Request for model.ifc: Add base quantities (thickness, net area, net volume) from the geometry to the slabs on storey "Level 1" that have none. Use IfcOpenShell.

First a look at what the model holds.

```python
import ifcopenshell
import ifcopenshell.util.element
import ifcopenshell.util.unit

model = ifcopenshell.open("model.ifc")
print(model.schema)
for unit_type in ("LENGTHUNIT", "AREAUNIT", "VOLUMEUNIT"):
    print(unit_type, ifcopenshell.util.unit.calculate_unit_scale(model, unit_type))
storey = next(s for s in model.by_type("IfcBuildingStorey") if s.Name == "Level 1")
slabs = [e for e in ifcopenshell.util.element.get_decomposition(storey) if e.is_a("IfcSlab")]
for e in sorted(slabs, key=lambda e: e.id()):
    print(e.id(), e.is_a(), e.Name, list(ifcopenshell.util.element.get_psets(e, qtos_only=True)), sep=" | ")
```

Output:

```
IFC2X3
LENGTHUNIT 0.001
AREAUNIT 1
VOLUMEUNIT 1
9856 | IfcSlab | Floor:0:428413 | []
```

```python
import ifcopenshell
import ifcopenshell.api.pset
import ifcopenshell.geom
import ifcopenshell.util.element
import ifcopenshell.util.shape
import ifcopenshell.util.unit

model = ifcopenshell.open("model.ifc")
unit_scale = ifcopenshell.util.unit.calculate_unit_scale(model)
area_scale = ifcopenshell.util.unit.calculate_unit_scale(model, "AREAUNIT")
volume_scale = ifcopenshell.util.unit.calculate_unit_scale(model, "VOLUMEUNIT")
settings = ifcopenshell.geom.settings()

storey = next(s for s in model.by_type("IfcBuildingStorey") if s.Name == "Level 1")
slabs = [e for e in ifcopenshell.util.element.get_decomposition(storey) if e.is_a("IfcSlab")]

for e in sorted(slabs, key=lambda e: e.id()):
    if ifcopenshell.util.element.get_psets(e, qtos_only=True, should_inherit=False):
        continue
    # Geometry comes back in metres, in the element's own axes.
    shape = ifcopenshell.geom.create_shape(settings, e)
    values = {
        "Width": ifcopenshell.util.shape.get_z(shape.geometry) / unit_scale,
        "NetArea": ifcopenshell.util.shape.get_footprint_area(shape.geometry) / area_scale,
        "NetVolume": ifcopenshell.util.shape.get_volume(shape.geometry) / volume_scale,
    }
    qto = ifcopenshell.api.pset.add_qto(model, product=e, name="BaseQuantities")
    ifcopenshell.api.pset.edit_qto(model, qto=qto, properties=values)
    print(e.id(), {k: round(v, 3) for k, v in values.items()})

model.write("model_updated.ifc")
```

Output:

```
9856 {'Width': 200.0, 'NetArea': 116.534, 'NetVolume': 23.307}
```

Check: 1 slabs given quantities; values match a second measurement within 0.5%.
